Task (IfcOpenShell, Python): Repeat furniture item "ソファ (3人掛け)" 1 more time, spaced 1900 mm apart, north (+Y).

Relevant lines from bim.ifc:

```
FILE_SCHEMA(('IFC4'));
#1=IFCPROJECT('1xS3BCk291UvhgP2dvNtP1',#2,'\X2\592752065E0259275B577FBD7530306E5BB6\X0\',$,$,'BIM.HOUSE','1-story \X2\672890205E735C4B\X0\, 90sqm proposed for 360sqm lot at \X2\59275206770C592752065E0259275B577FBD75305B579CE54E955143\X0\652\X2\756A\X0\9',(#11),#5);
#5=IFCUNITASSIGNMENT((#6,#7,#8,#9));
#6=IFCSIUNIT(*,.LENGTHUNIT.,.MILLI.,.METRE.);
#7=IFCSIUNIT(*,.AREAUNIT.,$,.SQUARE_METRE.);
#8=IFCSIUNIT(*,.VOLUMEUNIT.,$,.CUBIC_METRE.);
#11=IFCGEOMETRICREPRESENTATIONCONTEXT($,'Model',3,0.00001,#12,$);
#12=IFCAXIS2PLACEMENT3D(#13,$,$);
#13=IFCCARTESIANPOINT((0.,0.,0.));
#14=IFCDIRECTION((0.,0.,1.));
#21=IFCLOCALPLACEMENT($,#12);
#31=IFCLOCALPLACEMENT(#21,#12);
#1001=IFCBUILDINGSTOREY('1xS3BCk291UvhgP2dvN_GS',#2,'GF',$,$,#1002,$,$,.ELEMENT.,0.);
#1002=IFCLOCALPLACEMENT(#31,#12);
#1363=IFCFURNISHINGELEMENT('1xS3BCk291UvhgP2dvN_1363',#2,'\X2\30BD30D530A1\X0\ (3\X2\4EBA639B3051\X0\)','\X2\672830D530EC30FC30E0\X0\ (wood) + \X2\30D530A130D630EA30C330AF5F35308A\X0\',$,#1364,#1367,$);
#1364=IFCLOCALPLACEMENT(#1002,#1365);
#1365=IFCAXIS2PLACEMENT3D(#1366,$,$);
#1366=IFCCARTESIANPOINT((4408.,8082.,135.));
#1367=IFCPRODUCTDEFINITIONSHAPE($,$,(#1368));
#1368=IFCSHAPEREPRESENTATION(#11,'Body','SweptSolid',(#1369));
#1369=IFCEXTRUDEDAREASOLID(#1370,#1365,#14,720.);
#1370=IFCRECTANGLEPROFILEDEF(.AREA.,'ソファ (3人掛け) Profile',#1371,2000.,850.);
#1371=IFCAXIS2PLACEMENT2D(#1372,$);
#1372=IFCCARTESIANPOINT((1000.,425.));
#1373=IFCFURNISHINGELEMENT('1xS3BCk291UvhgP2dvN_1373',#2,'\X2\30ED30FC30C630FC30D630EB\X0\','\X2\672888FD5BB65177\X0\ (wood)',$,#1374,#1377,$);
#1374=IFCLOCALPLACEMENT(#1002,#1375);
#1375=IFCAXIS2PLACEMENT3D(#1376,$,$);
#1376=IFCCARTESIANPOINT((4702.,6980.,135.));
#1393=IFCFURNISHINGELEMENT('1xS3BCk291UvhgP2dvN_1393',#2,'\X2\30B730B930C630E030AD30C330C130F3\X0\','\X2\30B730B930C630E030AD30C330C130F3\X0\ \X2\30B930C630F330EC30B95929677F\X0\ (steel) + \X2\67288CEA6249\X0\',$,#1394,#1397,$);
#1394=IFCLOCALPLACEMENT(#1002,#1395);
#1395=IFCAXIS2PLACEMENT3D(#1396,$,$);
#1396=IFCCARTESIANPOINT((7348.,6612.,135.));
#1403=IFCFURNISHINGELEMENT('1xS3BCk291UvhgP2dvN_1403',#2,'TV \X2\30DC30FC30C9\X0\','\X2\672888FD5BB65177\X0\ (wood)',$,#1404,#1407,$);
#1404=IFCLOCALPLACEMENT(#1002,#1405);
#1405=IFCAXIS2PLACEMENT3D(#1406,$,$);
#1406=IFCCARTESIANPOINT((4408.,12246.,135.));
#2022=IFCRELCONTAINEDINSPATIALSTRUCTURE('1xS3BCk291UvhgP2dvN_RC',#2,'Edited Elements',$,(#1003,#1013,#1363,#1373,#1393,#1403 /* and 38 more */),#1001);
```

```python
import numpy as np
import ifcopenshell
import ifcopenshell.api.geometry
import ifcopenshell.api.root
import ifcopenshell.util.element
import ifcopenshell.util.placement
import ifcopenshell.util.unit

model = ifcopenshell.open("bim.ifc")
unit_scale = ifcopenshell.util.unit.calculate_unit_scale(model)


def reuse_history(source, copy):
    """copy_class also copies each property set's owner history, people and application; keep the originals."""
    for rel in copy.IsDefinedBy:
        if rel.is_a("IfcRelDefinesByProperties") and (history := rel.RelatingPropertyDefinition.OwnerHistory):
            rel.RelatingPropertyDefinition.OwnerHistory = source.OwnerHistory
            ifcopenshell.util.element.remove_deep2(model, history)


source = model.by_guid("1xS3BCk291UvhgP2dvN_1363")
base = ifcopenshell.util.placement.get_local_placement(source.ObjectPlacement)
step = np.array([0.0, 1.0, 0.0]) * 1.9 / unit_scale

for i in range(1, 2):
    copy = ifcopenshell.api.root.copy_class(model, product=source)
    copy.Representation = ifcopenshell.util.element.copy_deep(
        model, source.Representation, exclude=["IfcGeometricRepresentationContext", "IfcRepresentationMap"]
    )
    reuse_history(source, copy)
    matrix = base.copy()
    matrix[:3, 3] += i * step
    print("added at", matrix[:3, 3].round(3) + 0.0)
    ifcopenshell.api.geometry.edit_object_placement(model, product=copy, matrix=matrix, is_si=False)

model.write("bim_rev.ifc")
```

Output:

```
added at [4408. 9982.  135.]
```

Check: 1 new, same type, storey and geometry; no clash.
